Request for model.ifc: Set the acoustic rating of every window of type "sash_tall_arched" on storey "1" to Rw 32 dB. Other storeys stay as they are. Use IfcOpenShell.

First a look at what the model holds.

```python
import ifcopenshell
import ifcopenshell.util.element

model = ifcopenshell.open("model.ifc")
print(model.schema)
storey = next(s for s in model.by_type("IfcBuildingStorey") if s.Name == "1")
windows = [e for e in ifcopenshell.util.element.get_decomposition(storey) if e.is_a("IfcWindow")]
seen = {}
for e in windows:
    element_type = ifcopenshell.util.element.get_type(e)
    key = (element_type.Name if element_type != e and element_type else None, ifcopenshell.util.element.get_pset(e, "Pset_WindowCommon", "AcousticRating"))
    seen[key] = seen.get(key, 0) + 1
for (name, value), count in sorted(seen.items(), key=str):
    print(count, "x", name, "|", value)
```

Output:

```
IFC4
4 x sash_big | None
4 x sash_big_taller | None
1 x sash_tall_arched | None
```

```python
import ifcopenshell
import ifcopenshell.api.pset
import ifcopenshell.util.element

model = ifcopenshell.open("model.ifc")

storey = next(s for s in model.by_type("IfcBuildingStorey") if s.Name == "1")
windows = [e for e in ifcopenshell.util.element.get_decomposition(storey) if e.is_a("IfcWindow")]

count = 0
for e in windows:
    element_type = ifcopenshell.util.element.get_type(e)
    if element_type in (None, e) or element_type.Name != "sash_tall_arched":
        continue
    # add_pset returns the element's existing set when there is one.
    pset = ifcopenshell.api.pset.add_pset(model, product=e, name="Pset_WindowCommon")
    ifcopenshell.api.pset.edit_pset(model, pset=pset, properties={"AcousticRating": "Rw 32 dB"})
    count += 1

print(count, "windows updated")

model.write("model-out.ifc")
```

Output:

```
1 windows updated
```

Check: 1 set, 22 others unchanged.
